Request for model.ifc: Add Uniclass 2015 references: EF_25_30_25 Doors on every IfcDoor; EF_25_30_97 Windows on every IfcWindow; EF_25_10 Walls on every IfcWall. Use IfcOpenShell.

First a look at what the model holds.

```python
import ifcopenshell

model = ifcopenshell.open("model.ifc")
print(model.schema)
print("classifications:", [c.Name for c in model.by_type("IfcClassification")])
for ifc_class in ("IfcDoor", "IfcRoof", "IfcStair", "IfcWall", "IfcWindow"):
    print(ifc_class, len(model.by_type(ifc_class)))
```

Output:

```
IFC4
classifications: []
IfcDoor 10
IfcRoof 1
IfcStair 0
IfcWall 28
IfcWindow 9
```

```python
import ifcopenshell
import ifcopenshell.api.classification

model = ifcopenshell.open("model.ifc")

system = ifcopenshell.api.classification.add_classification(model, classification="Uniclass 2015")

codes = {
    "IfcDoor": ("EF_25_30_25", "Doors"),
    "IfcWindow": ("EF_25_30_97", "Windows"),
    "IfcWall": ("EF_25_10", "Walls"),
}
for ifc_class, (code, name) in codes.items():
    products = model.by_type(ifc_class)
    ifcopenshell.api.classification.add_reference(
        model, products=products, classification=system, identification=code, name=name
    )
    print(code, len(products))

model.write("model_edited.ifc")
```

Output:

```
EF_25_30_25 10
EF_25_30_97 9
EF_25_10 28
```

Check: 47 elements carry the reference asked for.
